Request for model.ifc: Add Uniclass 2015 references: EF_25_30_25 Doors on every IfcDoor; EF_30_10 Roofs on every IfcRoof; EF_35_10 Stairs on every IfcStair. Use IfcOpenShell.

First a look at what the model holds.

```python
import ifcopenshell

model = ifcopenshell.open("model.ifc")
print(model.schema)
print("classifications:", [c.Name for c in model.by_type("IfcClassification")])
for ifc_class in ("IfcDoor", "IfcRoof", "IfcStair", "IfcWall", "IfcWindow"):
    print(ifc_class, len(model.by_type(ifc_class)))
```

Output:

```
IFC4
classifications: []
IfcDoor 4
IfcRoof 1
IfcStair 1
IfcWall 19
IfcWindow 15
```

```python
import ifcopenshell
import ifcopenshell.api.classification

model = ifcopenshell.open("model.ifc")

system = ifcopenshell.api.classification.add_classification(model, classification="Uniclass 2015")

codes = {
    "IfcDoor": ("EF_25_30_25", "Doors"),
    "IfcRoof": ("EF_30_10", "Roofs"),
    "IfcStair": ("EF_35_10", "Stairs"),
}
for ifc_class, (code, name) in codes.items():
    products = model.by_type(ifc_class)
    ifcopenshell.api.classification.add_reference(
        model, products=products, classification=system, identification=code, name=name
    )
    print(code, len(products))

model.write("model_updated.ifc")
```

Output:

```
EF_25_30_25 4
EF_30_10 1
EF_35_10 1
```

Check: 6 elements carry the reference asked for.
